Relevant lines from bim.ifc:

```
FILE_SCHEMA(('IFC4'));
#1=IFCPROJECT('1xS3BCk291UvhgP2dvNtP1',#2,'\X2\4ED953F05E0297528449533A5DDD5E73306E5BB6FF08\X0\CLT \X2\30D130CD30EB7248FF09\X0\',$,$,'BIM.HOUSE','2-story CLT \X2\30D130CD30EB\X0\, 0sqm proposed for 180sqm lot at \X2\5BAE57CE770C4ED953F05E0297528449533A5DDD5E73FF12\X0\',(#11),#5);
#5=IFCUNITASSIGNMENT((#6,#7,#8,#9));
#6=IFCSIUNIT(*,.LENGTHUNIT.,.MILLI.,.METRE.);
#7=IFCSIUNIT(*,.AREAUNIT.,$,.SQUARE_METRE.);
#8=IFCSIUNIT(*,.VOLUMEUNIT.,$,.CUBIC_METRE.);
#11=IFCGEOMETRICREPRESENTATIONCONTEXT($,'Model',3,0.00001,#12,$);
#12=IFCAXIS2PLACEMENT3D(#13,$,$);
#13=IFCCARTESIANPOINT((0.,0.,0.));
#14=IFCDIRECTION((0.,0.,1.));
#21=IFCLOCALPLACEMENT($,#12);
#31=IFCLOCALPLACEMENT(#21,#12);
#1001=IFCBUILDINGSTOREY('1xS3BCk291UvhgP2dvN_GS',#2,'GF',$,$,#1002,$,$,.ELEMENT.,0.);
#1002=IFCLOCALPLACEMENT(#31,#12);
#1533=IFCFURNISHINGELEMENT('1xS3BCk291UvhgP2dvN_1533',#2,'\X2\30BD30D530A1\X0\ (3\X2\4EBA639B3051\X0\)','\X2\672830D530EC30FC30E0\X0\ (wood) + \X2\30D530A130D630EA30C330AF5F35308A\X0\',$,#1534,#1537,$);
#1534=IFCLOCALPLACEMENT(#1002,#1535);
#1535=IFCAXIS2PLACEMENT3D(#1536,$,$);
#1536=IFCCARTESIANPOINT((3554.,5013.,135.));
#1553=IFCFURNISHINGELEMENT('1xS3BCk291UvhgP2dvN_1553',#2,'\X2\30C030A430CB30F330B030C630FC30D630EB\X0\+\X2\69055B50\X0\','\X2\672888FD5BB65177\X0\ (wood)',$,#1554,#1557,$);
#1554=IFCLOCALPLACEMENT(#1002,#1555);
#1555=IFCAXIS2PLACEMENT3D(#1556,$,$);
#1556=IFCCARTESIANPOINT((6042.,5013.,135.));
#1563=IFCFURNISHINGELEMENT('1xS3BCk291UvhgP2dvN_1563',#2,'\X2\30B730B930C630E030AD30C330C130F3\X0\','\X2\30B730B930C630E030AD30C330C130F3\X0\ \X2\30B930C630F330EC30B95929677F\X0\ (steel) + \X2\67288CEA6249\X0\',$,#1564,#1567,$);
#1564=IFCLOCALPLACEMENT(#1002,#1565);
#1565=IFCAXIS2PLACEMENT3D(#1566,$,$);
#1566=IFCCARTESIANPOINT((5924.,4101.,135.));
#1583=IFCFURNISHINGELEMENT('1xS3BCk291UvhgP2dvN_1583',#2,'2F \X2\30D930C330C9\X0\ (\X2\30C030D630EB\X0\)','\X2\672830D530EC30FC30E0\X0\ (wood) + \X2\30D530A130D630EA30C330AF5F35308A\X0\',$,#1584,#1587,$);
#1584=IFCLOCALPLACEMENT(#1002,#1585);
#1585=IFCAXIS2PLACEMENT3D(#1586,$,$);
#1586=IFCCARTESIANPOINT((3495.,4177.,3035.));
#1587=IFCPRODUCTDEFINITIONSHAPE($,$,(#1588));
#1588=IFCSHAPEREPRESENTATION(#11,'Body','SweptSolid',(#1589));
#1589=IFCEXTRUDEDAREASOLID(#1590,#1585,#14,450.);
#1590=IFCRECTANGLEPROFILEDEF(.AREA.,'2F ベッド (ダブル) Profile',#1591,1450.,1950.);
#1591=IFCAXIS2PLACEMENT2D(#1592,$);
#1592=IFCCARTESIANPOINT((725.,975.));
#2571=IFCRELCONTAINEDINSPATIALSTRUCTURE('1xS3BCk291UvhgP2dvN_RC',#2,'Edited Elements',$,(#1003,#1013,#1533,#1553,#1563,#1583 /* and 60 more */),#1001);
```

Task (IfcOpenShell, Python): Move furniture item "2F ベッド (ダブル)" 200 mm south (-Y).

```python
import ifcopenshell
import ifcopenshell.api.geometry
import ifcopenshell.util.placement
import ifcopenshell.util.unit

model = ifcopenshell.open("bim.ifc")
unit_scale = ifcopenshell.util.unit.calculate_unit_scale(model)

item = model.by_guid("1xS3BCk291UvhgP2dvN_1583")
matrix = ifcopenshell.util.placement.get_local_placement(item.ObjectPlacement)
matrix[1, 3] -= 0.2 / unit_scale
ifcopenshell.api.geometry.edit_object_placement(model, product=item, matrix=matrix, is_si=False)

print(ifcopenshell.util.placement.get_local_placement(item.ObjectPlacement).round(3) + 0.0)

model.write("bim_updated.ifc")
```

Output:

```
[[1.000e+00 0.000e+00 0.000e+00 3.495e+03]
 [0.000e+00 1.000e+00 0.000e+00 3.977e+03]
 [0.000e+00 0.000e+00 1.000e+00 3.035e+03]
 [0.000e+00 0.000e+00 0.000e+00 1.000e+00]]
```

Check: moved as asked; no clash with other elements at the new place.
